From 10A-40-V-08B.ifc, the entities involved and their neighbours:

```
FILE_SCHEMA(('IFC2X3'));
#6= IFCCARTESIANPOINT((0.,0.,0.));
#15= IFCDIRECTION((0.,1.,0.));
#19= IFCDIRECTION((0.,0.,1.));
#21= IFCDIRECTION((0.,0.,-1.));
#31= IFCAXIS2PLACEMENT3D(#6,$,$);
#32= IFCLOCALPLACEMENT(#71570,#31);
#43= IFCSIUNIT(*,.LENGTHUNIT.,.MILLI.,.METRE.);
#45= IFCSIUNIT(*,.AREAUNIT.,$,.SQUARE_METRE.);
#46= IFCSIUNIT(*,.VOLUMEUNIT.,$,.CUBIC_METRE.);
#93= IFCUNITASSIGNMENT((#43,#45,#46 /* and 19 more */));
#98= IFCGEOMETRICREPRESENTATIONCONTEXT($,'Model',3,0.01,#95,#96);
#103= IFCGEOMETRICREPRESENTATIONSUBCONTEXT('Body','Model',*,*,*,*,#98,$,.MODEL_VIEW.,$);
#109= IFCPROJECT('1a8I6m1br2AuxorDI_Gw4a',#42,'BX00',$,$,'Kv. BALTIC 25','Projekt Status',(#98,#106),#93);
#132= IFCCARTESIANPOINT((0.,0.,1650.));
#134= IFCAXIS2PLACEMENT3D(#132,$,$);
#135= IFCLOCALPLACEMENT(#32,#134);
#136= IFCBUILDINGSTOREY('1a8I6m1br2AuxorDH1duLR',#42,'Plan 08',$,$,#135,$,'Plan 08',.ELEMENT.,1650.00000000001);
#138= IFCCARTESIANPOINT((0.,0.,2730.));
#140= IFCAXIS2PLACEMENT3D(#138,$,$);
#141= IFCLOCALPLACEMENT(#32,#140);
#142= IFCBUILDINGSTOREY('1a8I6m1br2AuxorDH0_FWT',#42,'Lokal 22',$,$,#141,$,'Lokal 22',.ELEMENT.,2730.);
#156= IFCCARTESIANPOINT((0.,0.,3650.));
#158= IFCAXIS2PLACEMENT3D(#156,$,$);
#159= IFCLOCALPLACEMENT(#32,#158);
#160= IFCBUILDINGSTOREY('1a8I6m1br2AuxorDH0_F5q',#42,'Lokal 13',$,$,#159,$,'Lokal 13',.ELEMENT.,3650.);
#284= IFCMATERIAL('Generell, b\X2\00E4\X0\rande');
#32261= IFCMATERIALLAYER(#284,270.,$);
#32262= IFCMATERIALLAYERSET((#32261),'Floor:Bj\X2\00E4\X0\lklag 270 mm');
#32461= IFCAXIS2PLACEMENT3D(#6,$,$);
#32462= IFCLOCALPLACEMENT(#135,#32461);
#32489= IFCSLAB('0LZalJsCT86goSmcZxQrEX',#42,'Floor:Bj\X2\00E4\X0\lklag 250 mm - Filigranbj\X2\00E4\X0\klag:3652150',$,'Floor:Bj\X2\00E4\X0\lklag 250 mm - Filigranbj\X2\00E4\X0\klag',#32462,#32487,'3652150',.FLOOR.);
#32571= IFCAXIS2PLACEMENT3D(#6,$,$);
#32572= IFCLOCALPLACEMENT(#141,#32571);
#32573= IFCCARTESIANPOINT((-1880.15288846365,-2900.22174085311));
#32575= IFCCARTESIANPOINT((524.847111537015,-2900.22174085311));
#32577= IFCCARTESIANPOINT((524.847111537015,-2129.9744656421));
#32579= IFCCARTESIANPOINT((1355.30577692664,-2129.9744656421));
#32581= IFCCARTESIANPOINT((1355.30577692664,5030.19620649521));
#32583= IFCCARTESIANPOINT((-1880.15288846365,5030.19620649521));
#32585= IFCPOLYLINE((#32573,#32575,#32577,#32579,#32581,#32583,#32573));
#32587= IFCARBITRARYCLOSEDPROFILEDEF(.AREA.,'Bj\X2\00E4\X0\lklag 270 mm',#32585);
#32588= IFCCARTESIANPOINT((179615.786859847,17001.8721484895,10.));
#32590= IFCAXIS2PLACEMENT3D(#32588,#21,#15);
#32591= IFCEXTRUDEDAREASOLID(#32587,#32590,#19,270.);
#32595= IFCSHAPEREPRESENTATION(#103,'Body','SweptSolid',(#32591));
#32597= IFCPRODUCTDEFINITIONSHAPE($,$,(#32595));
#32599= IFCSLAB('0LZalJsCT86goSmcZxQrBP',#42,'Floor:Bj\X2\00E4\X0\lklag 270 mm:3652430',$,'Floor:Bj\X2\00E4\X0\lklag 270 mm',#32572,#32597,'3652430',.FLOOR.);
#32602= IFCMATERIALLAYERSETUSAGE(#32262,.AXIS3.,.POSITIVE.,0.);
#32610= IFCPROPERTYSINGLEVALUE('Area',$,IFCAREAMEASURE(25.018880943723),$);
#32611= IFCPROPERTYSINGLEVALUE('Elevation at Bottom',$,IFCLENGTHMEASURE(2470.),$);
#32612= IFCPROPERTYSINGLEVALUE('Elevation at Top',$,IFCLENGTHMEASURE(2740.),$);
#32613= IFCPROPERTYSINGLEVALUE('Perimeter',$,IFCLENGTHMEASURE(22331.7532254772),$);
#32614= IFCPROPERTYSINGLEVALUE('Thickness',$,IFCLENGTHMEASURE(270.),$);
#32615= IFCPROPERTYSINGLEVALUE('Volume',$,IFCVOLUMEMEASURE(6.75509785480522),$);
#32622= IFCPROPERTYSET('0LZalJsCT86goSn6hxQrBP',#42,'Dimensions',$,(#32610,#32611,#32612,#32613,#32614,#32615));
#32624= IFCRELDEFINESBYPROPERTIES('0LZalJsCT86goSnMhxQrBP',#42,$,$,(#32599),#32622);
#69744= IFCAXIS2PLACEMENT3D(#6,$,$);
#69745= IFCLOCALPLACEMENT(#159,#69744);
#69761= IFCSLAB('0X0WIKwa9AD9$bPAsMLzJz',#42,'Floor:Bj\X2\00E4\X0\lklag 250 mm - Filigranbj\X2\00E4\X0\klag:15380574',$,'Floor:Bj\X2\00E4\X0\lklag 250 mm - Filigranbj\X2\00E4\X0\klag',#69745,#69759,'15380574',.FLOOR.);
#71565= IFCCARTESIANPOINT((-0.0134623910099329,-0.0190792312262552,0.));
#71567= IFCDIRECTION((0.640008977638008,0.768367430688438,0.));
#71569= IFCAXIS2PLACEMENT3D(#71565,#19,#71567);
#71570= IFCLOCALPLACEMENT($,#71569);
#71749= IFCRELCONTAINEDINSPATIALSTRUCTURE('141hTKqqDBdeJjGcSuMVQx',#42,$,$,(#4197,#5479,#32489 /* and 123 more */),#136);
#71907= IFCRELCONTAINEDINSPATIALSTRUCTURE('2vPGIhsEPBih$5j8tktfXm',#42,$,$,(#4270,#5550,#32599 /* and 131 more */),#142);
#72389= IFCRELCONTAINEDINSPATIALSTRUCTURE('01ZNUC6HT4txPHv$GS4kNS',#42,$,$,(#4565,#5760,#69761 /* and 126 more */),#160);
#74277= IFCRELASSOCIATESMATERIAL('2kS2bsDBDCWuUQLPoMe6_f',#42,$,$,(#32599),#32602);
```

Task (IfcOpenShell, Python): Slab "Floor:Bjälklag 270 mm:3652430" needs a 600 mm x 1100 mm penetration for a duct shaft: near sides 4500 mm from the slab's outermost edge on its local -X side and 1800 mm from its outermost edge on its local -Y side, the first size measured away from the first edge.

```python
import numpy as np
import ifcopenshell
import ifcopenshell.api.feature
import ifcopenshell.api.geometry
import ifcopenshell.api.pset
import ifcopenshell.api.root
import ifcopenshell.geom
import ifcopenshell.util.element
import ifcopenshell.util.placement
import ifcopenshell.util.representation
import ifcopenshell.util.shape
import ifcopenshell.util.unit

model = ifcopenshell.open("10A-40-V-08B.ifc")
unit_scale = ifcopenshell.util.unit.calculate_unit_scale(model)
area_scale = ifcopenshell.util.unit.calculate_unit_scale(model, "AREAUNIT")
volume_scale = ifcopenshell.util.unit.calculate_unit_scale(model, "VOLUMEUNIT")
settings = ifcopenshell.geom.settings()


def volume(element):
    """Net volume in cubic metres, openings subtracted."""
    shape = ifcopenshell.geom.create_shape(settings, element)
    return ifcopenshell.util.shape.get_volume(shape.geometry)


slab = model.by_guid("0LZalJsCT86goSmcZxQrBP")
before = volume(slab)

# Extent in the slab's own axes, in metres. The edges named are its -X and -Y sides.
slab_shape = ifcopenshell.geom.create_shape(settings, slab)
vertices = ifcopenshell.util.shape.get_vertices(slab_shape.geometry)
x_min, y_min, bottom = vertices.min(axis=0)
top = vertices[:, 2].max()

opening = ifcopenshell.api.root.create_entity(model, ifc_class="IfcOpeningElement", name="Duct shaft opening")
context = ifcopenshell.util.representation.get_context(model, "Model", "Body", "MODEL_VIEW")
width, depth = 0.6, 1.1
outline = [(0.0, 0.0), (width, 0.0), (width, depth), (0.0, depth), (0.0, 0.0)]
# Overshoot both faces by 50 mm so the cut is clean.
shape = ifcopenshell.api.geometry.add_slab_representation(
    model, context=context, depth=top - bottom + 0.1, polyline=outline
)
ifcopenshell.api.geometry.assign_representation(model, product=opening, representation=shape)

matrix = ifcopenshell.util.placement.get_local_placement(slab.ObjectPlacement)
matrix[:, 3] = matrix @ np.append(np.array([x_min + 4.5, y_min + 1.8, bottom - 0.05]) / unit_scale, 1.0)
ifcopenshell.api.geometry.edit_object_placement(model, product=opening, matrix=matrix, is_si=False)
ifcopenshell.api.feature.add_feature(model, feature=opening, element=slab)

after = volume(slab)

# Update the slab's stored quantities.
pset = model.by_id(ifcopenshell.util.element.get_pset(slab, "Dimensions", should_inherit=False)["id"])
ifcopenshell.api.pset.edit_pset(model, pset=pset, properties={
    "Area": model.create_entity("IfcAreaMeasure", after / (top - bottom) / area_scale),
    "Volume": model.create_entity("IfcVolumeMeasure", after / volume_scale),
})

print(f"slab volume {before:.3f} -> {after:.3f} m3")

model.write("10A-40-V-08B_v2.ifc")
```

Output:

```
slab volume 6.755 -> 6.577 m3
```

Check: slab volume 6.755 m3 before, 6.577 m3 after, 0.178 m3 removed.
